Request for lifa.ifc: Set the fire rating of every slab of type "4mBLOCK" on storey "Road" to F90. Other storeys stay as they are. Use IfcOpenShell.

First a look at what the model holds.

```python
import ifcopenshell
import ifcopenshell.util.element

model = ifcopenshell.open("lifa.ifc")
print(model.schema)
storey = next(s for s in model.by_type("IfcBuildingStorey") if s.Name == "Road")
slabs = [e for e in ifcopenshell.util.element.get_decomposition(storey) if e.is_a("IfcSlab")]
seen = {}
for e in slabs:
    element_type = ifcopenshell.util.element.get_type(e)
    key = (element_type.Name if element_type != e and element_type else None, ifcopenshell.util.element.get_pset(e, "Pset_SlabCommon", "FireRating"))
    seen[key] = seen.get(key, 0) + 1
for (name, value), count in sorted(seen.items(), key=str):
    print(count, "x", name, "|", value)
```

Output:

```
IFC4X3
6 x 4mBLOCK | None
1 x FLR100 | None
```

```python
import ifcopenshell
import ifcopenshell.api.pset
import ifcopenshell.util.element

model = ifcopenshell.open("lifa.ifc")

storey = next(s for s in model.by_type("IfcBuildingStorey") if s.Name == "Road")
slabs = [e for e in ifcopenshell.util.element.get_decomposition(storey) if e.is_a("IfcSlab")]

count = 0
for e in slabs:
    element_type = ifcopenshell.util.element.get_type(e)
    if element_type in (None, e) or element_type.Name != "4mBLOCK":
        continue
    # add_pset returns the element's existing set when there is one.
    pset = ifcopenshell.api.pset.add_pset(model, product=e, name="Pset_SlabCommon")
    ifcopenshell.api.pset.edit_pset(model, pset=pset, properties={"FireRating": "F90"})
    count += 1

print(count, "slabs updated")

model.write("lifa_edited.ifc")
```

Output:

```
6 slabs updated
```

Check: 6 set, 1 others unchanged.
